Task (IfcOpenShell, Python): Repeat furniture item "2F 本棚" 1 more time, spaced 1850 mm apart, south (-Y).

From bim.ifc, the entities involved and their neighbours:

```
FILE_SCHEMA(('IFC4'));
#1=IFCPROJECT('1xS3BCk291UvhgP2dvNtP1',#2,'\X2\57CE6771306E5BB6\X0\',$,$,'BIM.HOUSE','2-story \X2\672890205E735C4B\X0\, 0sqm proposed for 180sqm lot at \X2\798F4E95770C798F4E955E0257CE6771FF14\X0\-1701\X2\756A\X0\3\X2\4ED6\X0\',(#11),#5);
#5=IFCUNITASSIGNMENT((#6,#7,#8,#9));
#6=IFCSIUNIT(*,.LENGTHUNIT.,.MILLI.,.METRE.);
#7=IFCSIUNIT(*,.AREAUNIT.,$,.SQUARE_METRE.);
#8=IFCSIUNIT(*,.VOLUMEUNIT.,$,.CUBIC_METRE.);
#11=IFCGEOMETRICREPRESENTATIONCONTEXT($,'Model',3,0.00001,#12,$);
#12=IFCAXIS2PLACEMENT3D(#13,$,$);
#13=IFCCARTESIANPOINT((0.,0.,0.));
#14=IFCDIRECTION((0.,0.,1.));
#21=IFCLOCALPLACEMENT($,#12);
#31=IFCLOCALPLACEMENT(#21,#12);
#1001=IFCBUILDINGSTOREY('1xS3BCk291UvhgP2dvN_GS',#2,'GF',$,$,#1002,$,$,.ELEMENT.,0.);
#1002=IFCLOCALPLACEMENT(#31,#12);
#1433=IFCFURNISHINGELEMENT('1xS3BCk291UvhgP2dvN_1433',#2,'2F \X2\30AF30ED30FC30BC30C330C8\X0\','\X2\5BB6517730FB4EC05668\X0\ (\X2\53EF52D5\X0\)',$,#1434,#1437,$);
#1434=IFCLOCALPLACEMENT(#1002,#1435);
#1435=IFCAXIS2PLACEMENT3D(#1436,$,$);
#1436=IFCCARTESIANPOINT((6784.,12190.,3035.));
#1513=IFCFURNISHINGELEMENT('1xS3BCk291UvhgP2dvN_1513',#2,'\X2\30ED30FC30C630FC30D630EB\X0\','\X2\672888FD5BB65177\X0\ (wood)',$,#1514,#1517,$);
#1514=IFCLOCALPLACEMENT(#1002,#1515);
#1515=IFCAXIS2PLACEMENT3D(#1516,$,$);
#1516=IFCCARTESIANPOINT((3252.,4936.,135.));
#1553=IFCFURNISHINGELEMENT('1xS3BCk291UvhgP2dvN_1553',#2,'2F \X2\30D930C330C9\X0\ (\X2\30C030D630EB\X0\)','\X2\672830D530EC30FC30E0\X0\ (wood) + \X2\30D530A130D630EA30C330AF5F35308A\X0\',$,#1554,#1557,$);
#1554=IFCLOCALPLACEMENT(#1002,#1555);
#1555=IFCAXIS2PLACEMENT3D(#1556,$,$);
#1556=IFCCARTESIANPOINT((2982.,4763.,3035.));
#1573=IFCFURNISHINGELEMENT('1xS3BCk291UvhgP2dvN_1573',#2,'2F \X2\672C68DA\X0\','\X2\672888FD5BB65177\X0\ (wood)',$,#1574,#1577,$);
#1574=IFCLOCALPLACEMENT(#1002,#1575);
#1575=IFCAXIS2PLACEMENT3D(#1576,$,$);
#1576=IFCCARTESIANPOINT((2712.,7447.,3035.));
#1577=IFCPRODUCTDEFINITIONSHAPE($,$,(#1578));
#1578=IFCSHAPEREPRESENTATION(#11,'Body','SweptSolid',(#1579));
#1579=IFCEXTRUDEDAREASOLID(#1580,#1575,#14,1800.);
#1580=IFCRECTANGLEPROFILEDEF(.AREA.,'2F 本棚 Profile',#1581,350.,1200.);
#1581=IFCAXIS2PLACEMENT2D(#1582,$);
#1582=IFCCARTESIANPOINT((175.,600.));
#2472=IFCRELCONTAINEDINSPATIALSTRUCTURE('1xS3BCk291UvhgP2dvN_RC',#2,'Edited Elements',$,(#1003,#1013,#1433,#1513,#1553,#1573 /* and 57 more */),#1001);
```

```python
import numpy as np
import ifcopenshell
import ifcopenshell.api.geometry
import ifcopenshell.api.root
import ifcopenshell.util.element
import ifcopenshell.util.placement

model = ifcopenshell.open("bim.ifc")


def reuse_history(source, copy):
    """copy_class also copies each property set's owner history, people and application; keep the originals."""
    for rel in copy.IsDefinedBy:
        if rel.is_a("IfcRelDefinesByProperties") and (history := rel.RelatingPropertyDefinition.OwnerHistory):
            rel.RelatingPropertyDefinition.OwnerHistory = source.OwnerHistory
            ifcopenshell.util.element.remove_deep2(model, history)


source = model.by_id(1573)
base = ifcopenshell.util.placement.get_local_placement(source.ObjectPlacement)
step = np.array([0.0, -1.0, 0.0]) * 1850.0

for i in range(1, 2):
    copy = ifcopenshell.api.root.copy_class(model, product=source)
    copy.Representation = ifcopenshell.util.element.copy_deep(
        model, source.Representation, exclude=["IfcGeometricRepresentationContext", "IfcRepresentationMap"]
    )
    reuse_history(source, copy)
    matrix = base.copy()
    matrix[:3, 3] += i * step
    print("added at", matrix[:3, 3].round(3) + 0.0)
    ifcopenshell.api.geometry.edit_object_placement(model, product=copy, matrix=matrix, is_si=False)

model.write("bim-out.ifc")
```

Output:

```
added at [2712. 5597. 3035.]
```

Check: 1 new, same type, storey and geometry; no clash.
